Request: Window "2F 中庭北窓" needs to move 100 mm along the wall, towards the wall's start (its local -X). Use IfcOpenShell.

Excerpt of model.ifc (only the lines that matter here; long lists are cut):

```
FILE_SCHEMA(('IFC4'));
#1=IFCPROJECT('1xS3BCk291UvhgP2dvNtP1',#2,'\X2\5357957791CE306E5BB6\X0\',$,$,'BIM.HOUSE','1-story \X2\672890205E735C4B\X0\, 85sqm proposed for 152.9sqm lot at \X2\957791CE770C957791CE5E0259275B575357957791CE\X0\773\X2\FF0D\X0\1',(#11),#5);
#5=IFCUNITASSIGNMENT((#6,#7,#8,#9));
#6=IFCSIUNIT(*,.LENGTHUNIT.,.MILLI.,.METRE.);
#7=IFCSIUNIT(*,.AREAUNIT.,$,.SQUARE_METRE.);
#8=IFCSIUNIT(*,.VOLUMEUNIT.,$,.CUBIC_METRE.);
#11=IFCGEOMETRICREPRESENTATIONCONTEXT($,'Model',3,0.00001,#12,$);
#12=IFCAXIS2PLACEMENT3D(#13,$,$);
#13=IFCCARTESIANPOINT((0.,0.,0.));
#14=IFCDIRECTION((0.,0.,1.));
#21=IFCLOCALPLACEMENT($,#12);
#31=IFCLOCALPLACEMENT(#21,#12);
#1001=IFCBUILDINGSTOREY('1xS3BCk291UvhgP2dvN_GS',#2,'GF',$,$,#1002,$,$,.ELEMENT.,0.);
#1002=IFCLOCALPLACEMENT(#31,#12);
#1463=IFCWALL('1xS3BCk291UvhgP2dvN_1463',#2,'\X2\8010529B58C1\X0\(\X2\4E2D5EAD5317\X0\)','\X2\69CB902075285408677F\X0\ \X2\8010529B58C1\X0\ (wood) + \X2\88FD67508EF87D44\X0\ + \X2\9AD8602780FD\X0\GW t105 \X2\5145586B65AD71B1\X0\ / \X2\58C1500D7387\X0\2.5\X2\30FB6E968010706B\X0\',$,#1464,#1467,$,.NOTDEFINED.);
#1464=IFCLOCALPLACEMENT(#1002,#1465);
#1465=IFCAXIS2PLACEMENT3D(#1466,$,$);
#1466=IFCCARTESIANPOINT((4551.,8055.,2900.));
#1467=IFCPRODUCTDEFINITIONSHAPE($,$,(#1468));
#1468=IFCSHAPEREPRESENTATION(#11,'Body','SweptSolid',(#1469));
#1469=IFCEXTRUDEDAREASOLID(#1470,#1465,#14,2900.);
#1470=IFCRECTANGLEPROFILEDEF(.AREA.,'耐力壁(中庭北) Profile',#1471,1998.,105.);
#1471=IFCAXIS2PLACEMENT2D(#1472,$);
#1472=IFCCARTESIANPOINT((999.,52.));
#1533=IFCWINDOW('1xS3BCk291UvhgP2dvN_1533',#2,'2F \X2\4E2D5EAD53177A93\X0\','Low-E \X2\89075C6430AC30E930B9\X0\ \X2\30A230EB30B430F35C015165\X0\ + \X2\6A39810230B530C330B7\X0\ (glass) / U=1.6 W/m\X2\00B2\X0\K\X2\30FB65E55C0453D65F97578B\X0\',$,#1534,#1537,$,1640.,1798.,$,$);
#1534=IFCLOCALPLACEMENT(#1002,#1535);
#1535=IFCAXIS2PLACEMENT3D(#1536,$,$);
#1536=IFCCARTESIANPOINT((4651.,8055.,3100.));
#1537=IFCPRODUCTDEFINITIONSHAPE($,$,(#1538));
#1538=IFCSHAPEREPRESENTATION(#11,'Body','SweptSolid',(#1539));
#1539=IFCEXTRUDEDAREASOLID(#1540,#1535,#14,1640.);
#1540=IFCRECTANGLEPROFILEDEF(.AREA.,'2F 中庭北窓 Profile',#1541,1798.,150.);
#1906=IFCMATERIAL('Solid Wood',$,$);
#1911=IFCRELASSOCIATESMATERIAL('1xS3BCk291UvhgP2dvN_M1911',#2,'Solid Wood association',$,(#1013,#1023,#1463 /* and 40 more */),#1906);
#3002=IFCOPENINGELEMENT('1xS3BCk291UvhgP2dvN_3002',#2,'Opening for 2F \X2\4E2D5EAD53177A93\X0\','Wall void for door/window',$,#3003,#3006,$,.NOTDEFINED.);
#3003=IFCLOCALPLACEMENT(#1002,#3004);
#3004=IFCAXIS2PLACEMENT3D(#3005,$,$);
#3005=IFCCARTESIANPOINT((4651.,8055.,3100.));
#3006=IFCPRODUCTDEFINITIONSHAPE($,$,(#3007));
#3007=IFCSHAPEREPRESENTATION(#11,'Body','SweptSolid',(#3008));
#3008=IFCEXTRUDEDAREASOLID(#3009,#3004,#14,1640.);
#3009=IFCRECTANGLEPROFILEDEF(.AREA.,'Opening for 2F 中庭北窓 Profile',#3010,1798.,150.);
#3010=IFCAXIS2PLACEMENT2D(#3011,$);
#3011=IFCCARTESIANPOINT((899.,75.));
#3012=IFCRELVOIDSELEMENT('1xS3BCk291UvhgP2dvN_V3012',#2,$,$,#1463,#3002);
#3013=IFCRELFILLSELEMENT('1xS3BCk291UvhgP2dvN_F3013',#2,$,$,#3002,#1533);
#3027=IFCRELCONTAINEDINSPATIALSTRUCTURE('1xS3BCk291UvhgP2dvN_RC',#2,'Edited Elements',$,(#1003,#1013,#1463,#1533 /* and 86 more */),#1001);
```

```python
import ifcopenshell
import ifcopenshell.api.geometry
import ifcopenshell.util.placement
import ifcopenshell.util.unit

model = ifcopenshell.open("model.ifc")
unit_scale = ifcopenshell.util.unit.calculate_unit_scale(model)

window = model.by_id(1533)
opening = window.FillsVoids[0].RelatingOpeningElement
wall = opening.VoidsElements[0].RelatingBuildingElement

wall_matrix = ifcopenshell.util.placement.get_local_placement(wall.ObjectPlacement)
shift = wall_matrix[:3, 0] * -0.1 / unit_scale
before = ifcopenshell.util.placement.get_local_placement(window.ObjectPlacement)[:3, 3].copy()

# The window is not placed relative to its opening, so move both.
for product in (opening, window):
    matrix = ifcopenshell.util.placement.get_local_placement(product.ObjectPlacement)
    matrix[:3, 3] += shift
    ifcopenshell.api.geometry.edit_object_placement(model, product=product, matrix=matrix, is_si=False)

after = ifcopenshell.util.placement.get_local_placement(window.ObjectPlacement)[:3, 3]
print("window moved by", (after - before).round(3) + 0.0)

model.write("model_rev.ifc")
```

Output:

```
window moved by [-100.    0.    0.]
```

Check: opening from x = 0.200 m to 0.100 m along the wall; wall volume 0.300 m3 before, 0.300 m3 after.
